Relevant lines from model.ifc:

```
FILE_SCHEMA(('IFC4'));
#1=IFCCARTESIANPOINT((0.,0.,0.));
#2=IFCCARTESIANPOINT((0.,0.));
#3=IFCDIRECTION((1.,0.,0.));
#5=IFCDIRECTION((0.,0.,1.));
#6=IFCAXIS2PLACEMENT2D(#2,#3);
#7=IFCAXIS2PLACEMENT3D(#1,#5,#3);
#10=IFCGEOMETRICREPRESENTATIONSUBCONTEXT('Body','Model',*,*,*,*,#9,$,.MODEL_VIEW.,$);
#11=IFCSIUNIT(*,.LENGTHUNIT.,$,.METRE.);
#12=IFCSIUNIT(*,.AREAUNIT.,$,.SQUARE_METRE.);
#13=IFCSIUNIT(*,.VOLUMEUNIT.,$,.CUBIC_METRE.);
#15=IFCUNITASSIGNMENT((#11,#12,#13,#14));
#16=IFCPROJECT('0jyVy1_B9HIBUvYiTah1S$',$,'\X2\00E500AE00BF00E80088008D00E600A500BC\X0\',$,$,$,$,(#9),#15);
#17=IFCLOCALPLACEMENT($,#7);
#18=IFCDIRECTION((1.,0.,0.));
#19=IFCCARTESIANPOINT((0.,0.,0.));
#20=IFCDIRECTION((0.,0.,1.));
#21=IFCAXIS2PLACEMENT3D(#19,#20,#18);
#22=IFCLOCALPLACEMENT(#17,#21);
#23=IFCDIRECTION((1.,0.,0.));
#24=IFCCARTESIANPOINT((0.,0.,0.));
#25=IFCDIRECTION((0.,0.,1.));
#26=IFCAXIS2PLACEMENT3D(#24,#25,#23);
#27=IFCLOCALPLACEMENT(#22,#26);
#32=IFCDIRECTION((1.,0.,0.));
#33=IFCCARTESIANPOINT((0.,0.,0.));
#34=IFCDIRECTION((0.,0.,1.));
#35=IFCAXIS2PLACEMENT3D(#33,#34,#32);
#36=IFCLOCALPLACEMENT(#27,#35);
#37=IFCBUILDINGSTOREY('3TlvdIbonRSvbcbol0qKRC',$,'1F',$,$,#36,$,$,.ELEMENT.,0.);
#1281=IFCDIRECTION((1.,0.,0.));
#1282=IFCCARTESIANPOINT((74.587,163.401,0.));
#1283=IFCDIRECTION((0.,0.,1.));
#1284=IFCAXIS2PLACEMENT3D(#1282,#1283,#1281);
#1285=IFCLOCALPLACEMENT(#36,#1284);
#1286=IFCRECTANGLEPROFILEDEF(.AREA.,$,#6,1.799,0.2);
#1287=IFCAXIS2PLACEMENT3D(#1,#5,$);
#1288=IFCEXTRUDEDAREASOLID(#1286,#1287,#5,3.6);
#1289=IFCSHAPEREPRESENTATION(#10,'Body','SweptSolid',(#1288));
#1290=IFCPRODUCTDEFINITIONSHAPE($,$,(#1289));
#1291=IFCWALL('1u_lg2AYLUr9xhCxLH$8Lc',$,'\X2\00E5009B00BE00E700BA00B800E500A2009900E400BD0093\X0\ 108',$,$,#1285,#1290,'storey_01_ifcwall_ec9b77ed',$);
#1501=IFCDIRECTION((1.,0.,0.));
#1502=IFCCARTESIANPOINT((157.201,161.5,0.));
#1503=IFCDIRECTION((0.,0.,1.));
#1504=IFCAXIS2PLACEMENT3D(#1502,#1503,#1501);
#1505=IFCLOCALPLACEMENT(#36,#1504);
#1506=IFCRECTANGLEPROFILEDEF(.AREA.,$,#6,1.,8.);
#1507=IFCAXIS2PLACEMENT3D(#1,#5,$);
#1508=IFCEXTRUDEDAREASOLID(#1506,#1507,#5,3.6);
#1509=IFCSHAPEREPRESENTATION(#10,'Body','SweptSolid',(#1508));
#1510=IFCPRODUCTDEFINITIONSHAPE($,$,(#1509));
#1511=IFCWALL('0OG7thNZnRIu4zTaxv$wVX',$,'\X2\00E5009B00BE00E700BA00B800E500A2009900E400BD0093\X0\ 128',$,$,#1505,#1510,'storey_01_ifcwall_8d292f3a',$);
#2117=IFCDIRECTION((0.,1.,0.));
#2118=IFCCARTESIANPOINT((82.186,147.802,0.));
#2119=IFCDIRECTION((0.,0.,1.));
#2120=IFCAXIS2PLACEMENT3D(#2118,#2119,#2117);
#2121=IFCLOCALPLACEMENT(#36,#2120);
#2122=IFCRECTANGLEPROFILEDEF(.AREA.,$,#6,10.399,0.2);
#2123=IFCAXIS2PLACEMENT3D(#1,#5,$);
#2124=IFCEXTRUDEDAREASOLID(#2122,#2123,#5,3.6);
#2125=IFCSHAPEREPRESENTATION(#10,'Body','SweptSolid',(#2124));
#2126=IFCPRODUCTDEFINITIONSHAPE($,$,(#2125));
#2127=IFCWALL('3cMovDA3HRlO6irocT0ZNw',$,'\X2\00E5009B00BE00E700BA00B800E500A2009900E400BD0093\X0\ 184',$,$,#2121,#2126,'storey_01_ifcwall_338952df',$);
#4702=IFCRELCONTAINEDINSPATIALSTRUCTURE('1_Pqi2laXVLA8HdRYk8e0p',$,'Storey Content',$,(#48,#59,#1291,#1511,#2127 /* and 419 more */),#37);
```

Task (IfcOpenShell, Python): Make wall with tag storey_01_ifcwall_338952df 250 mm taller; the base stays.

```python
import ifcopenshell
import ifcopenshell.geom
import ifcopenshell.util.representation
import ifcopenshell.util.shape

model = ifcopenshell.open("model.ifc")
settings = ifcopenshell.geom.settings()


def volume(element):
    """Net volume in cubic metres, openings subtracted."""
    shape = ifcopenshell.geom.create_shape(settings, element)
    return ifcopenshell.util.shape.get_volume(shape.geometry)


wall = model.by_id(2127)
before = volume(wall)

body = ifcopenshell.util.representation.get_representation(wall, "Model", "Body")
solid = body.Items[0]
old_height = solid.Depth
solid.Depth += 0.25
after = volume(wall)

print(f"height {old_height:g} -> {solid.Depth:g}, volume {before:.3f} -> {after:.3f} m3")

model.write("model-out.ifc")
```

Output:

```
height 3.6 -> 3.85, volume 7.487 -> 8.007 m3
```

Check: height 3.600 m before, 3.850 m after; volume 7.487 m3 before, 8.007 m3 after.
